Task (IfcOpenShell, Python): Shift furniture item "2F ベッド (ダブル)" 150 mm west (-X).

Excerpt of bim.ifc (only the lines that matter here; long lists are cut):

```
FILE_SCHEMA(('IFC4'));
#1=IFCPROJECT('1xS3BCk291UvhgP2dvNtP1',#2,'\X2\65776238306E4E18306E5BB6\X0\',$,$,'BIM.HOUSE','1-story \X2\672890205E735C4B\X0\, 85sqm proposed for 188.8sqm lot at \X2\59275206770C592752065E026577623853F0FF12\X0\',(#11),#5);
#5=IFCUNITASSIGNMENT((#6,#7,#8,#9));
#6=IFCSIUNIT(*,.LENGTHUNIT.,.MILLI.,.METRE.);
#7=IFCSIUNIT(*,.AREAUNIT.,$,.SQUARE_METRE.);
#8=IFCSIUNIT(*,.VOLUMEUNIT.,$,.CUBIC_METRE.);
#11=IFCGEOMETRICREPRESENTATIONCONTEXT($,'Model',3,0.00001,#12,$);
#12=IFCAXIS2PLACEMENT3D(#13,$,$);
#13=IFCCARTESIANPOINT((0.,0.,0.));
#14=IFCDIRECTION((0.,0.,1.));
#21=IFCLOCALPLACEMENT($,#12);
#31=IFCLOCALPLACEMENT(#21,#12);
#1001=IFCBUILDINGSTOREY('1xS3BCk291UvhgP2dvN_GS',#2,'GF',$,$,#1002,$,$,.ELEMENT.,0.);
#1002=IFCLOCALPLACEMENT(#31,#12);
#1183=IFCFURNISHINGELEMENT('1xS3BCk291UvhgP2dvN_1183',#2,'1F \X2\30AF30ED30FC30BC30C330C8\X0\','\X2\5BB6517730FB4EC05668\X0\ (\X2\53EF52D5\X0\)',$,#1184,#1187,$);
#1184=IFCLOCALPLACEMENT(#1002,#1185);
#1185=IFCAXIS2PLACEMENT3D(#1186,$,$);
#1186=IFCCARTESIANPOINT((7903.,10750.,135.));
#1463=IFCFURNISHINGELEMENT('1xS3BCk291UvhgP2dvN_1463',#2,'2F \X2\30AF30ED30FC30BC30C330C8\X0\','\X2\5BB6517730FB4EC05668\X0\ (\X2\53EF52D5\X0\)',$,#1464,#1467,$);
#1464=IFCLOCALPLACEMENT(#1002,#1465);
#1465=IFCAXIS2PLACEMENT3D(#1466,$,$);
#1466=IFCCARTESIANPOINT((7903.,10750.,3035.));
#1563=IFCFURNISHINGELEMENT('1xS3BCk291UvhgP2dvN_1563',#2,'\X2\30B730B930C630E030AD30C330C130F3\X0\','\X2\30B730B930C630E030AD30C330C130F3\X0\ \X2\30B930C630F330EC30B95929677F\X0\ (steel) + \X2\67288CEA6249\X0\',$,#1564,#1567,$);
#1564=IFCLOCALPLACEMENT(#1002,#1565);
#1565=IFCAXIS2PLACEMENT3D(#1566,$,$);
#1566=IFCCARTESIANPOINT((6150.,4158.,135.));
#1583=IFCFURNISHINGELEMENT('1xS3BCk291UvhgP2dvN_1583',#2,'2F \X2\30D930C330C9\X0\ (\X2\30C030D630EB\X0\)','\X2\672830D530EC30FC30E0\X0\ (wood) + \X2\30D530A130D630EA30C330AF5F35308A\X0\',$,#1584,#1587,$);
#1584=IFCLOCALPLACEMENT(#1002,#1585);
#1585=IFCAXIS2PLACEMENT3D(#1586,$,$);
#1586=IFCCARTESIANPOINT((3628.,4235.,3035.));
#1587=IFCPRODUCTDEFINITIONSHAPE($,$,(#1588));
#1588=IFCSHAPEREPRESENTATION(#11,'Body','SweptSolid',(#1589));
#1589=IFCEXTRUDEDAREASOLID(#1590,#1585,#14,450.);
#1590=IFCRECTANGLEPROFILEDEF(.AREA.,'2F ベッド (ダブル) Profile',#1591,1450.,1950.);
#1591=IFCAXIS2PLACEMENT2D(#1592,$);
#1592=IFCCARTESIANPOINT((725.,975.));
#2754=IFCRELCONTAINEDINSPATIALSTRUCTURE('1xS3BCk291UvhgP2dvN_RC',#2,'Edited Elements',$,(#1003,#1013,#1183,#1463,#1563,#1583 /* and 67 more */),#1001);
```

```python
import ifcopenshell
import ifcopenshell.api.geometry
import ifcopenshell.util.placement
import ifcopenshell.util.unit

model = ifcopenshell.open("bim.ifc")
unit_scale = ifcopenshell.util.unit.calculate_unit_scale(model)

item = model.by_guid("1xS3BCk291UvhgP2dvN_1583")
matrix = ifcopenshell.util.placement.get_local_placement(item.ObjectPlacement)
matrix[0, 3] -= 0.15 / unit_scale
ifcopenshell.api.geometry.edit_object_placement(model, product=item, matrix=matrix, is_si=False)

print(ifcopenshell.util.placement.get_local_placement(item.ObjectPlacement).round(3) + 0.0)

model.write("bim_rev.ifc")
```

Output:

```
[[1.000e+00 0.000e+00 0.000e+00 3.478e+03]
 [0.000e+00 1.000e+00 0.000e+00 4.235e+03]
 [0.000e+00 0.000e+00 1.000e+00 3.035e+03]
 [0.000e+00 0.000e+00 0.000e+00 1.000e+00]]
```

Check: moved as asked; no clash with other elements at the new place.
